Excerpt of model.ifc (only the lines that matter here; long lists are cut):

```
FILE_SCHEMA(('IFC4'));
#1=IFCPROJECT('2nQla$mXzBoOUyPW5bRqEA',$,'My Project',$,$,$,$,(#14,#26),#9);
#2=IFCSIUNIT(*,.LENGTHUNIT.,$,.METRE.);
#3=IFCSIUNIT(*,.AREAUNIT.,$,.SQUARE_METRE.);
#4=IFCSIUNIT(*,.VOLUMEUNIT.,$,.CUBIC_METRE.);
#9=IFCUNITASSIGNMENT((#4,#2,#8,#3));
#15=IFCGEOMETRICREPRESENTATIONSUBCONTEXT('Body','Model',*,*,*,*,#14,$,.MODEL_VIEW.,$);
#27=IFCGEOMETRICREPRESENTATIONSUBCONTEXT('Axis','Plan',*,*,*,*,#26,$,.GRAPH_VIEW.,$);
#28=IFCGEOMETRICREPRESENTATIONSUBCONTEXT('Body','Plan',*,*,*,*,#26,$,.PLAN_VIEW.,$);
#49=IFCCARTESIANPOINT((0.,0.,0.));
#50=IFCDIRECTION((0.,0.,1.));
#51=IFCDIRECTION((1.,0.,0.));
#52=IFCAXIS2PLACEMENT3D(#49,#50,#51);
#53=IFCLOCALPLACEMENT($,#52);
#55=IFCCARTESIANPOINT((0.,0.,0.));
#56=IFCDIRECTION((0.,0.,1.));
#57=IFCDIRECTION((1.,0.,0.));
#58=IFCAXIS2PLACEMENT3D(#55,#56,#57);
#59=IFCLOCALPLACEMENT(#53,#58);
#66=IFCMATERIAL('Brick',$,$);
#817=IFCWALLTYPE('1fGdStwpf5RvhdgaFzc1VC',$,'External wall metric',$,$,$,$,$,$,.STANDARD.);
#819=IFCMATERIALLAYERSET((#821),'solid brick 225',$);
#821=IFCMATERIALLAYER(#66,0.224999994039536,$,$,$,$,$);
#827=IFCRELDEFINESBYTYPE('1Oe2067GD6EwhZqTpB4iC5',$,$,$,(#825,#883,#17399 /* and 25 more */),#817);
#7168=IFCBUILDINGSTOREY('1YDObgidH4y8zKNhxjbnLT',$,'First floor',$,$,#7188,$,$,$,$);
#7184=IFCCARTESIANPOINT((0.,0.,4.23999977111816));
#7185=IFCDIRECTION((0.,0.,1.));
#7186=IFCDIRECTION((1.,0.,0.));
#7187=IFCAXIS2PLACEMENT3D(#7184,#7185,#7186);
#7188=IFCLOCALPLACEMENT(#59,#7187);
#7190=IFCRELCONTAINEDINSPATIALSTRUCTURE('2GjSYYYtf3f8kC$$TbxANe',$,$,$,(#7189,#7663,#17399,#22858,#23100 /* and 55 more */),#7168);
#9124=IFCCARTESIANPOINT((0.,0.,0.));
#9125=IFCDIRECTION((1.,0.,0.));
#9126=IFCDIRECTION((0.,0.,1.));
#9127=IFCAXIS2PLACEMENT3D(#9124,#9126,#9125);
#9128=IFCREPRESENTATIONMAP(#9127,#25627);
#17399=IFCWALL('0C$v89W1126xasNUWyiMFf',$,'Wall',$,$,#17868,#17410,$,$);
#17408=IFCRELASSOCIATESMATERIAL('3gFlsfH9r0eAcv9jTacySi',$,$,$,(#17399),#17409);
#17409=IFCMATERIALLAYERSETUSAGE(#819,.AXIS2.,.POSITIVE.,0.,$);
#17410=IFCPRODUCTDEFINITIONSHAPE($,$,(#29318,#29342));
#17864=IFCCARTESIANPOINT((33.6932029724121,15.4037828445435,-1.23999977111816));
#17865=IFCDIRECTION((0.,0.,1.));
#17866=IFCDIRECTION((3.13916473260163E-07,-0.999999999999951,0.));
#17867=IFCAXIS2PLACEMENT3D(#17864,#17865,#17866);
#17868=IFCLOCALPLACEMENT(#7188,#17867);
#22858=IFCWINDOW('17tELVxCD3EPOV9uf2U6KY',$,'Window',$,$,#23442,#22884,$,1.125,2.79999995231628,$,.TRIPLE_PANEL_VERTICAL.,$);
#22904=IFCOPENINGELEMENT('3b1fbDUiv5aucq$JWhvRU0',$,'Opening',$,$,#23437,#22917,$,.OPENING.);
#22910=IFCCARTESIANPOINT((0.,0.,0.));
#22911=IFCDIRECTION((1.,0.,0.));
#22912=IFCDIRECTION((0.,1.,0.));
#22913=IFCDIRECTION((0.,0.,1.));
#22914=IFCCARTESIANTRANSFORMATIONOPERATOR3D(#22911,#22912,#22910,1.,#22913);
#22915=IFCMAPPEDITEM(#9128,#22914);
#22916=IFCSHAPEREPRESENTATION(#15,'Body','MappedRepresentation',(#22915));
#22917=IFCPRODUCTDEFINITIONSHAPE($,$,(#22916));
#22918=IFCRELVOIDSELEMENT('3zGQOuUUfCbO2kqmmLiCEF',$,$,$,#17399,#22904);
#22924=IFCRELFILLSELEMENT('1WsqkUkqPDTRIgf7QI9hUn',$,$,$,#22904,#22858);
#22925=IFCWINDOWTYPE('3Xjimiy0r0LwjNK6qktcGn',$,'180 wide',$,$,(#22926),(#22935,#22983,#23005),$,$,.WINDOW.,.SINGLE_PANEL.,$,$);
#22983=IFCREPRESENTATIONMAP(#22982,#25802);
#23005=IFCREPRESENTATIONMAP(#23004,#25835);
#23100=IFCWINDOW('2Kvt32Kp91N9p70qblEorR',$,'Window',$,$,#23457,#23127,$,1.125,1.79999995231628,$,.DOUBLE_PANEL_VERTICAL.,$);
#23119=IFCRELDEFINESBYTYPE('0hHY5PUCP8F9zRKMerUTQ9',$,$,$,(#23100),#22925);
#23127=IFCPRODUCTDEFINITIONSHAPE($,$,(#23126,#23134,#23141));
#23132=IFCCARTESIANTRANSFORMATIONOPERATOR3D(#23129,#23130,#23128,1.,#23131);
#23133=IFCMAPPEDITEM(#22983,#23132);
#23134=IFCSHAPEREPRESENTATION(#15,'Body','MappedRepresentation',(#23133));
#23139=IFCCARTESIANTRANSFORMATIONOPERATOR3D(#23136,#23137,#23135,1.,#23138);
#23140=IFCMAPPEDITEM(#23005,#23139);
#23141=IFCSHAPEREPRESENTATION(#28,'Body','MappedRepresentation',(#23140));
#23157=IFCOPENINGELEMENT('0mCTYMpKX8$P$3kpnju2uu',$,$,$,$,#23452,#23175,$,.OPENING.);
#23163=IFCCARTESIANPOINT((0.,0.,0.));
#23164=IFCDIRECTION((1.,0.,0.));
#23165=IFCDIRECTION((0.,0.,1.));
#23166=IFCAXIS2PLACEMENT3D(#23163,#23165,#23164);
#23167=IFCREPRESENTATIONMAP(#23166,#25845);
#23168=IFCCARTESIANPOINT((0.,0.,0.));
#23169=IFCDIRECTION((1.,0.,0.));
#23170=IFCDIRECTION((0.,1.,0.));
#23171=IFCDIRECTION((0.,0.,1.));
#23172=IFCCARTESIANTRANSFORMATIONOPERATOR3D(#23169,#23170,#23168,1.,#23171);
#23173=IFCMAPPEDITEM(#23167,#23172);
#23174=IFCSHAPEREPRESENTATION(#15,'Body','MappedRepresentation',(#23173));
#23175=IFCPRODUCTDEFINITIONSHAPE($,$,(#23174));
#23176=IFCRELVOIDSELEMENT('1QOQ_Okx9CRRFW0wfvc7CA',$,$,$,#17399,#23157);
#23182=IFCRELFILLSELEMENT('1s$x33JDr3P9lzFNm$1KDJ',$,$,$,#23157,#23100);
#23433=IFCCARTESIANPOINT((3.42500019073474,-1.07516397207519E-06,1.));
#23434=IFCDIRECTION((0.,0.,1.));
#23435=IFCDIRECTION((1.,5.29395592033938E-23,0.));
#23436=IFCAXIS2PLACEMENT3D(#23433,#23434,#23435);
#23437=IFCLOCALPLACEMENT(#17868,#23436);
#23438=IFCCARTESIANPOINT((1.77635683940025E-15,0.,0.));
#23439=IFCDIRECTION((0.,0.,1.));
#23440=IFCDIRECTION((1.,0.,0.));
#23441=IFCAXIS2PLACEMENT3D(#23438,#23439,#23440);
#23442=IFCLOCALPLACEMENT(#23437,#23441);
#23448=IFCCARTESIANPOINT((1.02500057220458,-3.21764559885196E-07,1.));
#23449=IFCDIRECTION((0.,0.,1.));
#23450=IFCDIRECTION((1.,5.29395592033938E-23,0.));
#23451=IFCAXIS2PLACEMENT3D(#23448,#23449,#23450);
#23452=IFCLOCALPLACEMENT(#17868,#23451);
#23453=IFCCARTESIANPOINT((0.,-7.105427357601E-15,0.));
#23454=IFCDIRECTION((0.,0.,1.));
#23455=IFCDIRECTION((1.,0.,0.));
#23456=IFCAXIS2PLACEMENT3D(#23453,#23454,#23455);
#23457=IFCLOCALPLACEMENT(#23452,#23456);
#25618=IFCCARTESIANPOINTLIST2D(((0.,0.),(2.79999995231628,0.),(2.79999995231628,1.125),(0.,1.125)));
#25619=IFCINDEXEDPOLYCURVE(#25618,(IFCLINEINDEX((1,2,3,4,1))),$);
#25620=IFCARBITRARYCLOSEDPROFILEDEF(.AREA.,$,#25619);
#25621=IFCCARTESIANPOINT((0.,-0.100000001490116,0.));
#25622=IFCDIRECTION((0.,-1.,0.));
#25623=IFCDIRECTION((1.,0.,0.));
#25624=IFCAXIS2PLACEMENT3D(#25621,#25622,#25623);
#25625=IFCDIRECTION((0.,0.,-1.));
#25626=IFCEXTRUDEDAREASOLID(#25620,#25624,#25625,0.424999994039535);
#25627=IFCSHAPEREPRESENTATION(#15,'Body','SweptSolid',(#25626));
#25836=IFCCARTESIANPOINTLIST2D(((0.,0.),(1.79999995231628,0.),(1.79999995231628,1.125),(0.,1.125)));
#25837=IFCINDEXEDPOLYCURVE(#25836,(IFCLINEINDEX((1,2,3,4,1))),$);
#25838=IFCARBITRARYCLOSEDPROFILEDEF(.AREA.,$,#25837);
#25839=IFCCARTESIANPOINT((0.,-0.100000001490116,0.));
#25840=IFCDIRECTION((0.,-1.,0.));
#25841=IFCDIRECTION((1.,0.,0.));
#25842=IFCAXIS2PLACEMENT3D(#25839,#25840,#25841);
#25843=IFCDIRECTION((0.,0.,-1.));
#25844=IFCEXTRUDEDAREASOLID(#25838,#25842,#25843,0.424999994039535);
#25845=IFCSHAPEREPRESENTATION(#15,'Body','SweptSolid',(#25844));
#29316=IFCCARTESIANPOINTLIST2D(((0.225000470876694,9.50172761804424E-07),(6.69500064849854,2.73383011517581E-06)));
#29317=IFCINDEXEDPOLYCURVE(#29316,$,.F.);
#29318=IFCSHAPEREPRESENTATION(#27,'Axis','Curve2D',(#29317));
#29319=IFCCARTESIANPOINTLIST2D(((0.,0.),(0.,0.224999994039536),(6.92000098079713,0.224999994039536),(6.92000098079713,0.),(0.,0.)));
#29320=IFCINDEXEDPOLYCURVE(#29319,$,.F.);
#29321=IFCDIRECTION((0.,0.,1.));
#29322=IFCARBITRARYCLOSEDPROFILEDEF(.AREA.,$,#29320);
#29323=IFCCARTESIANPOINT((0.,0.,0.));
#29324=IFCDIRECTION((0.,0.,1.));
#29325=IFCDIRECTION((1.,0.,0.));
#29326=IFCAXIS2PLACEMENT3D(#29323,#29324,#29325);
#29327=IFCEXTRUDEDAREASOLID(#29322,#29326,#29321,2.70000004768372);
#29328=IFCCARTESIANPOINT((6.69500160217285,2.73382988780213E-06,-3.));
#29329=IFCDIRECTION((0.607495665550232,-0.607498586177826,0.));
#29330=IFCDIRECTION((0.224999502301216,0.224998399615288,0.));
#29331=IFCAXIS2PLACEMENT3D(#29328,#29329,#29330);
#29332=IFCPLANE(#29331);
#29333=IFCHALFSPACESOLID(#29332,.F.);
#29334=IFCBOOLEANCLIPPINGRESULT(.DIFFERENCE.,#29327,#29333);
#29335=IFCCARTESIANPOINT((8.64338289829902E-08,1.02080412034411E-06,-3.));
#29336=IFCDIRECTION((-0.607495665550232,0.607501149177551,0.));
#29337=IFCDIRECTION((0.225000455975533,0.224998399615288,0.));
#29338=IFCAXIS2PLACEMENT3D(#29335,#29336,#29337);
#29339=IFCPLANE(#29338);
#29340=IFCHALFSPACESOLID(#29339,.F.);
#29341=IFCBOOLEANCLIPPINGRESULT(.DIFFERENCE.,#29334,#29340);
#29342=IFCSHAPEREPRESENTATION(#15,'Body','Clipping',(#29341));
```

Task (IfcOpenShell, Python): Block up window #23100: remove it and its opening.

```python
import ifcopenshell
import ifcopenshell.api.feature
import ifcopenshell.api.root
import ifcopenshell.geom
import ifcopenshell.util.shape

model = ifcopenshell.open("model.ifc")
settings = ifcopenshell.geom.settings()


def volume(element):
    """Net volume in cubic metres, openings subtracted."""
    shape = ifcopenshell.geom.create_shape(settings, element)
    return ifcopenshell.util.shape.get_volume(shape.geometry)


window = model.by_id(23100)
opening = window.FillsVoids[0].RelatingOpeningElement
wall = opening.VoidsElements[0].RelatingBuildingElement
before = volume(wall)

ifcopenshell.api.root.remove_product(model, product=window)
ifcopenshell.api.feature.remove_feature(model, feature=opening)

after = volume(wall)

print(f"wall volume {before:.3f} -> {after:.3f} m3")

model.write("model_updated.ifc")
```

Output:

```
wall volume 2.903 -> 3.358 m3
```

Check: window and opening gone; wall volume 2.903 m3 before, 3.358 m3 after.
